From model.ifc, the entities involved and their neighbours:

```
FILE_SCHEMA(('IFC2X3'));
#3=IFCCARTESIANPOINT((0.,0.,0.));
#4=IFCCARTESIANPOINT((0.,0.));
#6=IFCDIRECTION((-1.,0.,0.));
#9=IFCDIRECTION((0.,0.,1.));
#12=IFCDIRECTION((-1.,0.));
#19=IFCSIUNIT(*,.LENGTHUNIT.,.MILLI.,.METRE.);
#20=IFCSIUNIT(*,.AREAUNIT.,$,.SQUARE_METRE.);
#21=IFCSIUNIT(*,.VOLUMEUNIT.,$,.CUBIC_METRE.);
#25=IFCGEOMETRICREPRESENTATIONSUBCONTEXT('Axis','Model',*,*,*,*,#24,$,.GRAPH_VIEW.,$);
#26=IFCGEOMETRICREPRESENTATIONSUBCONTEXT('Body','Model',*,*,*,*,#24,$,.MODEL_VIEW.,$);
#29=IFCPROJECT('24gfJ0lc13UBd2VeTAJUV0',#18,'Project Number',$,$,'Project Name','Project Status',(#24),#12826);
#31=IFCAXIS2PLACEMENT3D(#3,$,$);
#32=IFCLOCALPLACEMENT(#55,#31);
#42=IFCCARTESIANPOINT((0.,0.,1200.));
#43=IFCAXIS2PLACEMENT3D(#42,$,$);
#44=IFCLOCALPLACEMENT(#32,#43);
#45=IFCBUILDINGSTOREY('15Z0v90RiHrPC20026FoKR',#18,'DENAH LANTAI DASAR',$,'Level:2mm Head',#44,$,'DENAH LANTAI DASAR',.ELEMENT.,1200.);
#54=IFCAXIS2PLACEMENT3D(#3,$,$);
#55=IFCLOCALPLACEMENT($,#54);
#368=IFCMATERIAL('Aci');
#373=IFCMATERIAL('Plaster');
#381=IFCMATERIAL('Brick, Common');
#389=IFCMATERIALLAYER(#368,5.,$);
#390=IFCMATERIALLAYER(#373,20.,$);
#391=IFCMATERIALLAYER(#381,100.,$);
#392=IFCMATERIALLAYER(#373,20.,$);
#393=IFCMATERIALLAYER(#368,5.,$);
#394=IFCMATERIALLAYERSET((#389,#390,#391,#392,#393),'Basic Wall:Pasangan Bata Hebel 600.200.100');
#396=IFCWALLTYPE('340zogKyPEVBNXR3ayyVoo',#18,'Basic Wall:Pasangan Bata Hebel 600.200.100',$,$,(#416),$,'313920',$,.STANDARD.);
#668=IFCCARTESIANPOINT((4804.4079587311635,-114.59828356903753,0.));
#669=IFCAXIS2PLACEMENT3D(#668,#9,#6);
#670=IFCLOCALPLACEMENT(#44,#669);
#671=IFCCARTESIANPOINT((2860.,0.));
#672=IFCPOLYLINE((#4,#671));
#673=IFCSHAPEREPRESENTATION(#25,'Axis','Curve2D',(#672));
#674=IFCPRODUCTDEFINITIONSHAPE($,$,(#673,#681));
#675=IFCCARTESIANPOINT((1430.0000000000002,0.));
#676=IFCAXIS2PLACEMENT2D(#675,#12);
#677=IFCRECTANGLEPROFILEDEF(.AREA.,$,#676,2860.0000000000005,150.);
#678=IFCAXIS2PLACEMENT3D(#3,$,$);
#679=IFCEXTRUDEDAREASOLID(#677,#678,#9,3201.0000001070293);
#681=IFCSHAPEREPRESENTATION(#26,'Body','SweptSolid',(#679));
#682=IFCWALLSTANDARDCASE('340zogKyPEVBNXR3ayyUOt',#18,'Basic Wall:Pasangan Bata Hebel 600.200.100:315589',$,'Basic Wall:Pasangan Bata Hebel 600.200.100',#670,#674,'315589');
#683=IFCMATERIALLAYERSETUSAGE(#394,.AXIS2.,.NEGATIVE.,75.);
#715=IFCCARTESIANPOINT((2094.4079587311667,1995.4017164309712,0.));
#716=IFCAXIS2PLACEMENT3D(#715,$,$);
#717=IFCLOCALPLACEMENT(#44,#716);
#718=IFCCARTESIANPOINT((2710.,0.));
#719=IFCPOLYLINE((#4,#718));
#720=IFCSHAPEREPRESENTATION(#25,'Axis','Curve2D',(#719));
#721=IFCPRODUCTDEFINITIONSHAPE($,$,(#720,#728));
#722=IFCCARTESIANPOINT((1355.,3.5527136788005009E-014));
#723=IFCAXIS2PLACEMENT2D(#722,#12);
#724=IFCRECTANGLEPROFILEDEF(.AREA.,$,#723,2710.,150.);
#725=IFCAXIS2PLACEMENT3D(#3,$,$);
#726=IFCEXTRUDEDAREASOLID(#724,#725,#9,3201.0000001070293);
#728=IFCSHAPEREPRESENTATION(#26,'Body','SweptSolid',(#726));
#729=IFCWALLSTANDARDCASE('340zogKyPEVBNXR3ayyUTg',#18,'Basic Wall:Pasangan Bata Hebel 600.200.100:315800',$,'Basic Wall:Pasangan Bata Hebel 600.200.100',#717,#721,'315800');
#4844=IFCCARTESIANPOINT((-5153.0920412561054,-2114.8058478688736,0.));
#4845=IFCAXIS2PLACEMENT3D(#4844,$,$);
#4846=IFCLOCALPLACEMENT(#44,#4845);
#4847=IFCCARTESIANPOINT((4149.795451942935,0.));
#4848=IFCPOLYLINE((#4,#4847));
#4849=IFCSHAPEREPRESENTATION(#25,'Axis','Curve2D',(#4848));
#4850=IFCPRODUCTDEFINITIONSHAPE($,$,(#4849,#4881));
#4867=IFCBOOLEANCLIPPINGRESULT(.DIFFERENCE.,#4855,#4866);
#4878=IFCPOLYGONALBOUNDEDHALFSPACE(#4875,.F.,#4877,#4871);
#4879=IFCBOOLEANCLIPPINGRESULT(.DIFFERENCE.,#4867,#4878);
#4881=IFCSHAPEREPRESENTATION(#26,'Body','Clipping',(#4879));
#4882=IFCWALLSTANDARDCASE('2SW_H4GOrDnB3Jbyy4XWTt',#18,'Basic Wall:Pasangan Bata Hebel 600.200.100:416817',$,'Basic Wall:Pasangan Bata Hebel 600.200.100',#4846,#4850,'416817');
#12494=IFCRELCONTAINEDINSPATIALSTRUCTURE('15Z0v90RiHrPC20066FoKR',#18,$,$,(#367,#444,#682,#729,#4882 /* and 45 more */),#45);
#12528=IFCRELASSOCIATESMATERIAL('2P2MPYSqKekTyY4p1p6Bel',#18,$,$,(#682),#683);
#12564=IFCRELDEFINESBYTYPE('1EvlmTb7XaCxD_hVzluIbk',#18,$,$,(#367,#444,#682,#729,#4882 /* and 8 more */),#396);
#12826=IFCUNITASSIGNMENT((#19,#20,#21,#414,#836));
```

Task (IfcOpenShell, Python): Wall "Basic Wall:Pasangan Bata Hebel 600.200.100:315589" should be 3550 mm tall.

```python
import ifcopenshell
import ifcopenshell.geom
import ifcopenshell.util.representation
import ifcopenshell.util.shape

model = ifcopenshell.open("model.ifc")
settings = ifcopenshell.geom.settings()


def volume(element):
    """Net volume in cubic metres, openings subtracted."""
    shape = ifcopenshell.geom.create_shape(settings, element)
    return ifcopenshell.util.shape.get_volume(shape.geometry)


wall = model.by_guid("340zogKyPEVBNXR3ayyUOt")
before = volume(wall)

body = ifcopenshell.util.representation.get_representation(wall, "Model", "Body")
solid = body.Items[0]
old_height = solid.Depth
solid.Depth = 3550.0
after = volume(wall)

print(f"height {old_height:g} -> {solid.Depth:g}, volume {before:.3f} -> {after:.3f} m3")

model.write("model-out.ifc")
```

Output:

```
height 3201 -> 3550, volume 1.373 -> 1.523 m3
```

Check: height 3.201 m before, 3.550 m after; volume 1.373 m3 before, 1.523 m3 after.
